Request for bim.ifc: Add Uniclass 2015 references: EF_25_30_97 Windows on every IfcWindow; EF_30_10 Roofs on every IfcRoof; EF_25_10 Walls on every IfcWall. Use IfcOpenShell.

First a look at what the model holds.

```python
import ifcopenshell

model = ifcopenshell.open("bim.ifc")
print(model.schema)
print("classifications:", [c.Name for c in model.by_type("IfcClassification")])
for ifc_class in ("IfcDoor", "IfcRoof", "IfcStair", "IfcWall", "IfcWindow"):
    print(ifc_class, len(model.by_type(ifc_class)))
```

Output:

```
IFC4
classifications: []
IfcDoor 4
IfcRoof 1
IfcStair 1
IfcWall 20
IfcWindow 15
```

```python
import ifcopenshell
import ifcopenshell.api.classification

model = ifcopenshell.open("bim.ifc")

system = ifcopenshell.api.classification.add_classification(model, classification="Uniclass 2015")

codes = {
    "IfcWindow": ("EF_25_30_97", "Windows"),
    "IfcRoof": ("EF_30_10", "Roofs"),
    "IfcWall": ("EF_25_10", "Walls"),
}
for ifc_class, (code, name) in codes.items():
    products = model.by_type(ifc_class)
    ifcopenshell.api.classification.add_reference(
        model, products=products, classification=system, identification=code, name=name
    )
    print(code, len(products))

model.write("bim_v2.ifc")
```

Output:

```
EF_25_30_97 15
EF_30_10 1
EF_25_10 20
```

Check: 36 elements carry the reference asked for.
